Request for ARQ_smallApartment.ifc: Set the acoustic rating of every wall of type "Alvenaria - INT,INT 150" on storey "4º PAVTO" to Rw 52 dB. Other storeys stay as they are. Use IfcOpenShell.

First a look at what the model holds.

```python
import ifcopenshell
import ifcopenshell.util.element

model = ifcopenshell.open("ARQ_smallApartment.ifc")
print(model.schema)
storey = next(s for s in model.by_type("IfcBuildingStorey") if s.Name == "4º PAVTO")
walls = [e for e in ifcopenshell.util.element.get_decomposition(storey) if e.is_a("IfcWall")]
seen = {}
for e in walls:
    element_type = ifcopenshell.util.element.get_type(e)
    key = (element_type.Name if element_type != e and element_type else None, ifcopenshell.util.element.get_pset(e, "Pset_WallCommon", "AcousticRating"))
    seen[key] = seen.get(key, 0) + 1
for (name, value), count in sorted(seen.items(), key=str):
    print(count, "x", name, "|", value)
```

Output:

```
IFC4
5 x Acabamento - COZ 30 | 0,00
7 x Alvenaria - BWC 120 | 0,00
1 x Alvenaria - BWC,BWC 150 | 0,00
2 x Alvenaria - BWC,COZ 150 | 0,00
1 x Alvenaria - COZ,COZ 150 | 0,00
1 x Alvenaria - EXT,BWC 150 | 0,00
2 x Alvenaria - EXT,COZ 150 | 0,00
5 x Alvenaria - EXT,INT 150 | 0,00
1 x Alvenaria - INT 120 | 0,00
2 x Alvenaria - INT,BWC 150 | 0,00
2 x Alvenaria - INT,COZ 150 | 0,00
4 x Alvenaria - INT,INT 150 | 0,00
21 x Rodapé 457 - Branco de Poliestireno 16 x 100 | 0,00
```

```python
import ifcopenshell
import ifcopenshell.api.pset
import ifcopenshell.util.element

model = ifcopenshell.open("ARQ_smallApartment.ifc")

storey = next(s for s in model.by_type("IfcBuildingStorey") if s.Name == "4º PAVTO")
walls = [e for e in ifcopenshell.util.element.get_decomposition(storey) if e.is_a("IfcWall")]

count = 0
for e in walls:
    element_type = ifcopenshell.util.element.get_type(e)
    if element_type in (None, e) or element_type.Name != "Alvenaria - INT,INT 150":
        continue
    # add_pset returns the element's existing set when there is one.
    pset = ifcopenshell.api.pset.add_pset(model, product=e, name="Pset_WallCommon")
    ifcopenshell.api.pset.edit_pset(model, pset=pset, properties={"AcousticRating": "Rw 52 dB"})
    count += 1

print(count, "walls updated")

model.write("ARQ_smallApartment-out.ifc")
```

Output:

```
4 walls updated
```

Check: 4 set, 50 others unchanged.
